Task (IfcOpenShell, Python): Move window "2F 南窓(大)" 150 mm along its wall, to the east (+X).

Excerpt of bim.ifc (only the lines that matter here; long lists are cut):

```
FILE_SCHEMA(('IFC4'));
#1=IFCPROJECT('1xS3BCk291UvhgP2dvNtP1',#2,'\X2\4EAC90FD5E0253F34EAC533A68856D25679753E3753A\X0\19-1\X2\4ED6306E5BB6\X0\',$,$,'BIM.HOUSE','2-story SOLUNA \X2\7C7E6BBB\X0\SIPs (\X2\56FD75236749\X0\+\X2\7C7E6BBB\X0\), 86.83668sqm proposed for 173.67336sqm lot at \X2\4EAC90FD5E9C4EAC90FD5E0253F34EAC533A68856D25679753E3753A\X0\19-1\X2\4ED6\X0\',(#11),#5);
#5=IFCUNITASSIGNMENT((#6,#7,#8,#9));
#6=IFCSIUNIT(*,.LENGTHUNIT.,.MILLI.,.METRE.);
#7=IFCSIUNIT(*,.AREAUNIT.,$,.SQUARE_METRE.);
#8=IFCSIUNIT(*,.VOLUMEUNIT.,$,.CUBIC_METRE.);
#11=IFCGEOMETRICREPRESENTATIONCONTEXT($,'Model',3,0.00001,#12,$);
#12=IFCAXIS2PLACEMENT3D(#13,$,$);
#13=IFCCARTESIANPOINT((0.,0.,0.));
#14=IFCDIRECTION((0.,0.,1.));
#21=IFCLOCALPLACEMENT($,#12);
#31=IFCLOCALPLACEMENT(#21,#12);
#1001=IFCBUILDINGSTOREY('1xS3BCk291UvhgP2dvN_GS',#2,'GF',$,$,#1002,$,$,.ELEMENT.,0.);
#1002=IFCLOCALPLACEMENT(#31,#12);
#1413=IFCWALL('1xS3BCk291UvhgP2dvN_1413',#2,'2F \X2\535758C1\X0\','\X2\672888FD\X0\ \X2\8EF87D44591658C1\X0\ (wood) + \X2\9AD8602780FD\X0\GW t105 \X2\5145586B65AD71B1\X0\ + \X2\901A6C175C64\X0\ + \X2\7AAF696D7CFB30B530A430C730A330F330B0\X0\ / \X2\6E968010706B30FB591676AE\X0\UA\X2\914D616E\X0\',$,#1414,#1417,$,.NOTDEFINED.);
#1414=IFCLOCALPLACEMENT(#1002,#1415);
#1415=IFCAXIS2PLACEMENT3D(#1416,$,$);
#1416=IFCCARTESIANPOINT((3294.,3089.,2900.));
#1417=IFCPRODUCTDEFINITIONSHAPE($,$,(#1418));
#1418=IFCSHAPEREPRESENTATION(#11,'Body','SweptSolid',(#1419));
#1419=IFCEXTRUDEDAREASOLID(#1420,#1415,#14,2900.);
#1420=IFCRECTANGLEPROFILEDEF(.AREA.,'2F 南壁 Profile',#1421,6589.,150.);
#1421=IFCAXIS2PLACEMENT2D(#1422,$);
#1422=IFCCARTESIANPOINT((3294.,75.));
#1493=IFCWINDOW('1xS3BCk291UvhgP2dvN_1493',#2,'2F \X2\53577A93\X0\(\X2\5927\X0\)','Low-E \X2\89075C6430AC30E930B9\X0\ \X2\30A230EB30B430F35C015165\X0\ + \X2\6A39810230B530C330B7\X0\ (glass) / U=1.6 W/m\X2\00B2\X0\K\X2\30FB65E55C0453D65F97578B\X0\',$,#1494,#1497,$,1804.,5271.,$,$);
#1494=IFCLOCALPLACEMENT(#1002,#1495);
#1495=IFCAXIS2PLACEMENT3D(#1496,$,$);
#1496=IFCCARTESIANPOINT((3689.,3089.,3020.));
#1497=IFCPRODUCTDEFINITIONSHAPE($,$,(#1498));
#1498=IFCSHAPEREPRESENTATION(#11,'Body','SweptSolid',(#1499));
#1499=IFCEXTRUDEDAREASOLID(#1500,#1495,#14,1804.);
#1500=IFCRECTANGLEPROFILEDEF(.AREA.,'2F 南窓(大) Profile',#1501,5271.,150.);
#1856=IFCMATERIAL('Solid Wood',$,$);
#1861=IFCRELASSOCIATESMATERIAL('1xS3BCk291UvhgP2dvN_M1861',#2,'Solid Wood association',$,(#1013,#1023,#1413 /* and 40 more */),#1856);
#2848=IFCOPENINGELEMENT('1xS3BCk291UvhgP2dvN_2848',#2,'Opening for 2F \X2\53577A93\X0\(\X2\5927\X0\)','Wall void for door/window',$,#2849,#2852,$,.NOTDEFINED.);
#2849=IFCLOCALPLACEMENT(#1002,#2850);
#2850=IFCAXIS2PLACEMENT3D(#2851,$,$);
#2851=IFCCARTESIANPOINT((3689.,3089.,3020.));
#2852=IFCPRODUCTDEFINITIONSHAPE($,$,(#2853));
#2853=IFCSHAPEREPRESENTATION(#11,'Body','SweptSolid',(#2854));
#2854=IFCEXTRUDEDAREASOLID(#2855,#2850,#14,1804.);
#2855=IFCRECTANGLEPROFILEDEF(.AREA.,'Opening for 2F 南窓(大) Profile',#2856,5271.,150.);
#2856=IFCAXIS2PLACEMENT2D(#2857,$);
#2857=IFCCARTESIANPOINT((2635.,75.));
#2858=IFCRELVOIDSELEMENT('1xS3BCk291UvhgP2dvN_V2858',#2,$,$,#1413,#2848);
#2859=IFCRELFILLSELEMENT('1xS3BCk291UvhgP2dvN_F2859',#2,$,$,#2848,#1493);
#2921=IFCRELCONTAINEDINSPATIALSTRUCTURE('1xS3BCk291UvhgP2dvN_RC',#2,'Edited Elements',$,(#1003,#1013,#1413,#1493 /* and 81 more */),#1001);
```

```python
import ifcopenshell
import ifcopenshell.api.geometry
import ifcopenshell.util.placement

model = ifcopenshell.open("bim.ifc")

window = model.by_guid("1xS3BCk291UvhgP2dvN_1493")
opening = window.FillsVoids[0].RelatingOpeningElement
wall = opening.VoidsElements[0].RelatingBuildingElement

wall_matrix = ifcopenshell.util.placement.get_local_placement(wall.ObjectPlacement)
shift = wall_matrix[:3, 0] * 150.0
before = ifcopenshell.util.placement.get_local_placement(window.ObjectPlacement)[:3, 3].copy()

# The window is not placed relative to its opening, so move both.
for product in (opening, window):
    matrix = ifcopenshell.util.placement.get_local_placement(product.ObjectPlacement)
    matrix[:3, 3] += shift
    ifcopenshell.api.geometry.edit_object_placement(model, product=product, matrix=matrix, is_si=False)

after = ifcopenshell.util.placement.get_local_placement(window.ObjectPlacement)[:3, 3]
print("window moved by", (after - before).round(3) + 0.0)

model.write("bim_updated.ifc")
```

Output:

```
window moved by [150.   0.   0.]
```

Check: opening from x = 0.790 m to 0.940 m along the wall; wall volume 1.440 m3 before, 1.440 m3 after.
